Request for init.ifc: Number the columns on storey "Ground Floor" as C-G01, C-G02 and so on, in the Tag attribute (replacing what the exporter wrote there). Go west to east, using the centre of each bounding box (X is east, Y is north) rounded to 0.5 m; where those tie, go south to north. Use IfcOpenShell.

First a look at what the model holds.

```python
import ifcopenshell
import ifcopenshell.util.element
import ifcopenshell.util.placement

model = ifcopenshell.open("init.ifc")
print(model.schema)
storey = next(s for s in model.by_type("IfcBuildingStorey") if s.Name == "Ground Floor")
columns = [e for e in ifcopenshell.util.element.get_decomposition(storey) if e.is_a("IfcColumn")]
for e in sorted(columns, key=lambda e: e.id()):
    origin = ifcopenshell.util.placement.get_local_placement(e.ObjectPlacement)[:3, 3]
    print(e.id(), e.Tag, e.Name, origin.round(2) + 0.0, sep=" | ")
```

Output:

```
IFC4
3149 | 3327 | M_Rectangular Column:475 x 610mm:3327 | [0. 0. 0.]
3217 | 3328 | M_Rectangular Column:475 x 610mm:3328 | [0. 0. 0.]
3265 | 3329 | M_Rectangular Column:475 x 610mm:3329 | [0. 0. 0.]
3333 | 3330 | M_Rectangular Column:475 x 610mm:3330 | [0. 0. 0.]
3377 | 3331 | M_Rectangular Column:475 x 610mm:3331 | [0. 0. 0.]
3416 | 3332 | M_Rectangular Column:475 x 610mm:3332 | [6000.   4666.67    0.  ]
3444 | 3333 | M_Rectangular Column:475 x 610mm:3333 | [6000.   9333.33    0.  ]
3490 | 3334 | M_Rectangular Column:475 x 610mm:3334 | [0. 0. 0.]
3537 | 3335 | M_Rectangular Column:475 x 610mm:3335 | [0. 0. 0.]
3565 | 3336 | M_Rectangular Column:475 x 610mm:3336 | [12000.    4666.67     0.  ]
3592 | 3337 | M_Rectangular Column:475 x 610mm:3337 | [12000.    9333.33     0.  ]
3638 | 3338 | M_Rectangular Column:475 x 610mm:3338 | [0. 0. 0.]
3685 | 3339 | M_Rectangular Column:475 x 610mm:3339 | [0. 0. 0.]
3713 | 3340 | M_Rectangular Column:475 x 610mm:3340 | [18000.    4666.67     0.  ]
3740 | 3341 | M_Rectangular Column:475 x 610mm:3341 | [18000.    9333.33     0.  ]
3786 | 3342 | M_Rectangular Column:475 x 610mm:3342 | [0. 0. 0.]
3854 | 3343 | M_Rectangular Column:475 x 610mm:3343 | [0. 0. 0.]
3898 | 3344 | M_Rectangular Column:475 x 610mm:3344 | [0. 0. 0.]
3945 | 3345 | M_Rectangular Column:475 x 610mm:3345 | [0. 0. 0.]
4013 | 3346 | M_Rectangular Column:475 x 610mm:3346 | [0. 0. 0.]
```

```python
import ifcopenshell
import ifcopenshell.geom
import ifcopenshell.util.element
import ifcopenshell.util.shape

model = ifcopenshell.open("init.ifc")
settings = ifcopenshell.geom.settings()
settings.set("use-world-coords", True)


def centre(element):
    shape = ifcopenshell.geom.create_shape(settings, element)
    return ifcopenshell.util.shape.get_bbox_centroid(shape.geometry)


storey = next(s for s in model.by_type("IfcBuildingStorey") if s.Name == "Ground Floor")
columns = [e for e in ifcopenshell.util.element.get_decomposition(storey) if e.is_a("IfcColumn")]

# Insertion points can sit at a corner or the storey origin, so sort by the geometry (in metres).
centres = {e: centre(e) for e in columns}
columns.sort(key=lambda e: (round(centres[e][0] / 0.5), centres[e][1]))

for i, e in enumerate(columns, start=1):
    number = f"C-G{i:02d}"
    e.Tag = number
    print(e.id(), number)

model.write("init-out.ifc")
```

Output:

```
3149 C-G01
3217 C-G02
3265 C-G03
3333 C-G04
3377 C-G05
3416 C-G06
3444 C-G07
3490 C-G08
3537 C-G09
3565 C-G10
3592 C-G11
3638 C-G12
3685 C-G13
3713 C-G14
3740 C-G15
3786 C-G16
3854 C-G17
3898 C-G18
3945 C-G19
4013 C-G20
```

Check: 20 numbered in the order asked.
